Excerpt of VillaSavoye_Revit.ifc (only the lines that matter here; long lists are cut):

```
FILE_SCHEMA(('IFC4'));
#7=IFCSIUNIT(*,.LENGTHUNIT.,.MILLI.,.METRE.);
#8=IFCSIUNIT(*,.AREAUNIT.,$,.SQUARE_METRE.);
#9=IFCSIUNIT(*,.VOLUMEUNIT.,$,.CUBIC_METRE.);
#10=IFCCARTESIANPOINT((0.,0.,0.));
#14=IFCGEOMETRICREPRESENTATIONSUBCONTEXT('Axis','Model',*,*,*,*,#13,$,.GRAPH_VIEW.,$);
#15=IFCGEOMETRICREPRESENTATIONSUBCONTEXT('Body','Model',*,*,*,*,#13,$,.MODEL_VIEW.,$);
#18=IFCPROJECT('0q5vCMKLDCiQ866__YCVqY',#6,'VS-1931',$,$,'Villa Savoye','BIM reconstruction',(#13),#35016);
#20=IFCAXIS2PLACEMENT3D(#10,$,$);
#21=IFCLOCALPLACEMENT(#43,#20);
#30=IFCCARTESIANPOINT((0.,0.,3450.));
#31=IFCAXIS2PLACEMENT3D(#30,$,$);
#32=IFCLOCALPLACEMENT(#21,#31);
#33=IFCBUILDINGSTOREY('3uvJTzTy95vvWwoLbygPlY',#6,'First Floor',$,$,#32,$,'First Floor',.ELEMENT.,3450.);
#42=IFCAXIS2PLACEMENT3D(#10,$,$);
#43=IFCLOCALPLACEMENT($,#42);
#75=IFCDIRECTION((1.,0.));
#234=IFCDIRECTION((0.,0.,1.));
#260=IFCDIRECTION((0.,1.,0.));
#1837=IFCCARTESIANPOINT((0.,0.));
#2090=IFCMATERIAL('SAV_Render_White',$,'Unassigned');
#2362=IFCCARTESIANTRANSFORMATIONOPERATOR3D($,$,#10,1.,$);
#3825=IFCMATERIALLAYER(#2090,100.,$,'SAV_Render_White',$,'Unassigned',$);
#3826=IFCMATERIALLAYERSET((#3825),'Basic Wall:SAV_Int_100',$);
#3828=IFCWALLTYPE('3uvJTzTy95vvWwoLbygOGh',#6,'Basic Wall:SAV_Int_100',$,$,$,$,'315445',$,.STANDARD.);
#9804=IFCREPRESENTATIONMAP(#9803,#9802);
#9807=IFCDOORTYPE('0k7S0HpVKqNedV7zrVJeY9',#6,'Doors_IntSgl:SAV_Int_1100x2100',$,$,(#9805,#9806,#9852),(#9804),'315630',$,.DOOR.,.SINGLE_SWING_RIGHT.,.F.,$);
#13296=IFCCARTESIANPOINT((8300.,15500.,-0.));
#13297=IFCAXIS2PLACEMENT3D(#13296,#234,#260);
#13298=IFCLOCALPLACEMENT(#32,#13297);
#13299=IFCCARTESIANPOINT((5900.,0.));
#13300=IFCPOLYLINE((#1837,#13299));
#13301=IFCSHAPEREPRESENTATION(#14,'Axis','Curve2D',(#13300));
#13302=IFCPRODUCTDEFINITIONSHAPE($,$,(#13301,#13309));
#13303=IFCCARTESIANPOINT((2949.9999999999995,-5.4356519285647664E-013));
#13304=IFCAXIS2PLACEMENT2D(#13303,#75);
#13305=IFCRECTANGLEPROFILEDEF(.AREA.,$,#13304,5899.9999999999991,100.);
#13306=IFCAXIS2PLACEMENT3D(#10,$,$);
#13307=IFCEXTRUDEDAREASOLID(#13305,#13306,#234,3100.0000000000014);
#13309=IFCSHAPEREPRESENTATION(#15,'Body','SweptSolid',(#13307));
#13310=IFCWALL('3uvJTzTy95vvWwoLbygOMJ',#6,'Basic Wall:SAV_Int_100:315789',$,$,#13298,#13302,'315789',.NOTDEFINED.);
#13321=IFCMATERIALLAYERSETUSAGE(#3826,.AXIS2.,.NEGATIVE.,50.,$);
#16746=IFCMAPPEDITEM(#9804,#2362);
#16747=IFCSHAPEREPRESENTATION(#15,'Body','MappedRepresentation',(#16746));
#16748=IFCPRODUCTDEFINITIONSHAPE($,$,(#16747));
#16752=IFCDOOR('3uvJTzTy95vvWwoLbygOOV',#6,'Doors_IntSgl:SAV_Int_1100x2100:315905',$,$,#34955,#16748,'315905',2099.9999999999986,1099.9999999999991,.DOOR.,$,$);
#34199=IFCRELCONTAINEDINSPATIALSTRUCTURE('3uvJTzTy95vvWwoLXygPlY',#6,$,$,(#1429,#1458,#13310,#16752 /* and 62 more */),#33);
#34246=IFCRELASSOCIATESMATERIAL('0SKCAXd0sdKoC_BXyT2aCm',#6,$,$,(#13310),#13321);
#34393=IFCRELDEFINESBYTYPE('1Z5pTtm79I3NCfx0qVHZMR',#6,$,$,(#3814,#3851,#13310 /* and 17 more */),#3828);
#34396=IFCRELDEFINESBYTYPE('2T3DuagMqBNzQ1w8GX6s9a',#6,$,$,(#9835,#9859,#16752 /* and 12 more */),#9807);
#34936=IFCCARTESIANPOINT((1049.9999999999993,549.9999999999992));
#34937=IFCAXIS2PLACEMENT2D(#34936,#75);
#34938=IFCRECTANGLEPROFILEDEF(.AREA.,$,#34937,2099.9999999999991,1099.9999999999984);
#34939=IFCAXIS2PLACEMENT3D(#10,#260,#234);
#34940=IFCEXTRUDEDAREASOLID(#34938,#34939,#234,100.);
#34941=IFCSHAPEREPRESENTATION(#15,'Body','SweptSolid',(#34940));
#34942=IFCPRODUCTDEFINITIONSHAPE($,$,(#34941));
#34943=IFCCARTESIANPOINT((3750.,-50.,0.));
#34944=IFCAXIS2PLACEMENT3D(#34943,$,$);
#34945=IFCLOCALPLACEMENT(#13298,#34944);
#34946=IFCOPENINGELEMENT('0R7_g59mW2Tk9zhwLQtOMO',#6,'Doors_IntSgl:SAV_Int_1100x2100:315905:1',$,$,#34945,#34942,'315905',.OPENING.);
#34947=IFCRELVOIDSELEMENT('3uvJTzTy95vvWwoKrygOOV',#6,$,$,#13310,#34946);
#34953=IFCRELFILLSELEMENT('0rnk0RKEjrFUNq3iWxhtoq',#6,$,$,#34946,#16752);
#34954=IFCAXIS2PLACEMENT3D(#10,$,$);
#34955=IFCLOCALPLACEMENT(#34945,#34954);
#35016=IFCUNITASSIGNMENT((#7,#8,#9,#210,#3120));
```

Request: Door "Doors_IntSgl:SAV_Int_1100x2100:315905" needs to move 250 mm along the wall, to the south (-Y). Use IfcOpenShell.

```python
import ifcopenshell
import ifcopenshell.api.geometry
import ifcopenshell.util.placement

model = ifcopenshell.open("VillaSavoye_Revit.ifc")

door = model.by_id(16752)
opening = door.FillsVoids[0].RelatingOpeningElement
wall = opening.VoidsElements[0].RelatingBuildingElement

wall_matrix = ifcopenshell.util.placement.get_local_placement(wall.ObjectPlacement)
shift = wall_matrix[:3, 0] * -250.0
before = ifcopenshell.util.placement.get_local_placement(door.ObjectPlacement)[:3, 3].copy()

# The door is placed relative to its opening, so it follows when the opening moves.
matrix = ifcopenshell.util.placement.get_local_placement(opening.ObjectPlacement)
matrix[:3, 3] += shift
ifcopenshell.api.geometry.edit_object_placement(
    model, product=opening, matrix=matrix, is_si=False, should_transform_children=True
)

after = ifcopenshell.util.placement.get_local_placement(door.ObjectPlacement)[:3, 3]
print("door moved by", (after - before).round(3) + 0.0)

model.write("VillaSavoye_Revit_v2.ifc")
```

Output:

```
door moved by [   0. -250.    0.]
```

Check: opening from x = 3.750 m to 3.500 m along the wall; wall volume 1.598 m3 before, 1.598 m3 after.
